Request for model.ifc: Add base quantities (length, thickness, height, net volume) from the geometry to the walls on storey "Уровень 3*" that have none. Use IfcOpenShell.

First a look at what the model holds.

```python
import ifcopenshell
import ifcopenshell.util.element
import ifcopenshell.util.unit

model = ifcopenshell.open("model.ifc")
print(model.schema)
for unit_type in ("LENGTHUNIT", "AREAUNIT", "VOLUMEUNIT"):
    print(unit_type, ifcopenshell.util.unit.calculate_unit_scale(model, unit_type))
storey = next(s for s in model.by_type("IfcBuildingStorey") if s.Name == "Уровень 3*")
walls = [e for e in ifcopenshell.util.element.get_decomposition(storey) if e.is_a("IfcWall")]
for e in sorted(walls, key=lambda e: e.id()):
    print(e.id(), e.is_a(), e.Name, list(ifcopenshell.util.element.get_psets(e, qtos_only=True)), sep=" | ")
```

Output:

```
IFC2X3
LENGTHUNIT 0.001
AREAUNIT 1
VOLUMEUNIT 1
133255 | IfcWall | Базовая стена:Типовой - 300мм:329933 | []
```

```python
import ifcopenshell
import ifcopenshell.api.pset
import ifcopenshell.geom
import ifcopenshell.util.element
import ifcopenshell.util.shape
import ifcopenshell.util.unit

model = ifcopenshell.open("model.ifc")
unit_scale = ifcopenshell.util.unit.calculate_unit_scale(model)
volume_scale = ifcopenshell.util.unit.calculate_unit_scale(model, "VOLUMEUNIT")
settings = ifcopenshell.geom.settings()

storey = next(s for s in model.by_type("IfcBuildingStorey") if s.Name == "Уровень 3*")
walls = [e for e in ifcopenshell.util.element.get_decomposition(storey) if e.is_a("IfcWall")]

for e in sorted(walls, key=lambda e: e.id()):
    if ifcopenshell.util.element.get_psets(e, qtos_only=True, should_inherit=False):
        continue
    # Geometry comes back in metres, in the element's own axes.
    shape = ifcopenshell.geom.create_shape(settings, e)
    values = {
        "Length": ifcopenshell.util.shape.get_x(shape.geometry) / unit_scale,
        "Width": ifcopenshell.util.shape.get_y(shape.geometry) / unit_scale,
        "Height": ifcopenshell.util.shape.get_z(shape.geometry) / unit_scale,
        "NetVolume": ifcopenshell.util.shape.get_volume(shape.geometry) / volume_scale,
    }
    qto = ifcopenshell.api.pset.add_qto(model, product=e, name="BaseQuantities")
    ifcopenshell.api.pset.edit_qto(model, qto=qto, properties=values)
    print(e.id(), {k: round(v, 3) for k, v in values.items()})

model.write("model_rev.ifc")
```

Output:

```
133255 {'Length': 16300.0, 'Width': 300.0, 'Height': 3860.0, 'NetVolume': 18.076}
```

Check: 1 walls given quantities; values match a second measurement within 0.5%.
